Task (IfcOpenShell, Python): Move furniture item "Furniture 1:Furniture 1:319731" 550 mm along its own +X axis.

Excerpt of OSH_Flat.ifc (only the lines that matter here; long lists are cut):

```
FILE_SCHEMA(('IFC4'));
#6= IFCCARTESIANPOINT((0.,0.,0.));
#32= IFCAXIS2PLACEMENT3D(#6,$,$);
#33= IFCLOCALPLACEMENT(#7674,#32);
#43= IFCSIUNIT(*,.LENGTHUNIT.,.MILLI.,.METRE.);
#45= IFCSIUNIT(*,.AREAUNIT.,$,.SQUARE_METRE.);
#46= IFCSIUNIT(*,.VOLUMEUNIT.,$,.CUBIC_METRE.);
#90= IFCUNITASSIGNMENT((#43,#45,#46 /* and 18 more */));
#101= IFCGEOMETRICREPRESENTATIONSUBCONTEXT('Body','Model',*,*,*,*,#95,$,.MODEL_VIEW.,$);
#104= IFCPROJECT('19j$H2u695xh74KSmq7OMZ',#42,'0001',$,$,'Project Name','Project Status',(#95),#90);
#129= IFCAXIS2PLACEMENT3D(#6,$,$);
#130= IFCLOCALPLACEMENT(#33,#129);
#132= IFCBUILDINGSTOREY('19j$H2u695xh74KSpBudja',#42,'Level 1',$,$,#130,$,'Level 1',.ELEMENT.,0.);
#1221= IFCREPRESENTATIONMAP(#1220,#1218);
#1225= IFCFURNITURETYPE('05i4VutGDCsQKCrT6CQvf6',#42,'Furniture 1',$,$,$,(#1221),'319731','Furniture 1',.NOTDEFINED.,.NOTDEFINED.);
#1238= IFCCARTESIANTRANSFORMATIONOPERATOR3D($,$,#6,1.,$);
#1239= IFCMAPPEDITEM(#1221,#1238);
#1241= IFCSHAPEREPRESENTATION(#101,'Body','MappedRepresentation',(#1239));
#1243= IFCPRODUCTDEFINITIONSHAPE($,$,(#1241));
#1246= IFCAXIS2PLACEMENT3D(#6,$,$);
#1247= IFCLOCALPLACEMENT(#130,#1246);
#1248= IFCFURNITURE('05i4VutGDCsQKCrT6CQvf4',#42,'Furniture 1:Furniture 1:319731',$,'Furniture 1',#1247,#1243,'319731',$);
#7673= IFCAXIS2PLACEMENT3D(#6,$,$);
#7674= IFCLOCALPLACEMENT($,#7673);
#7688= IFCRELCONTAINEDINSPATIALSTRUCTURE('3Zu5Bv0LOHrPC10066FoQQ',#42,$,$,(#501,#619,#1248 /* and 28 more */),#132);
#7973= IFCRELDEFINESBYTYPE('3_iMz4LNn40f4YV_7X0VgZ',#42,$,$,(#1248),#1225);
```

```python
import ifcopenshell
import ifcopenshell.api.geometry
import ifcopenshell.util.placement

model = ifcopenshell.open("OSH_Flat.ifc")

item = model.by_guid("05i4VutGDCsQKCrT6CQvf4")
matrix = ifcopenshell.util.placement.get_local_placement(item.ObjectPlacement)
matrix[:3, 3] += matrix[:3, 0] * 550.0
ifcopenshell.api.geometry.edit_object_placement(model, product=item, matrix=matrix, is_si=False)

print(ifcopenshell.util.placement.get_local_placement(item.ObjectPlacement).round(3) + 0.0)

model.write("OSH_Flat_v2.ifc")
```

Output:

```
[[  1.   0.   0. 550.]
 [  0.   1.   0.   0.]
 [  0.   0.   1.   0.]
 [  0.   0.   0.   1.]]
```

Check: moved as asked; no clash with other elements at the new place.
